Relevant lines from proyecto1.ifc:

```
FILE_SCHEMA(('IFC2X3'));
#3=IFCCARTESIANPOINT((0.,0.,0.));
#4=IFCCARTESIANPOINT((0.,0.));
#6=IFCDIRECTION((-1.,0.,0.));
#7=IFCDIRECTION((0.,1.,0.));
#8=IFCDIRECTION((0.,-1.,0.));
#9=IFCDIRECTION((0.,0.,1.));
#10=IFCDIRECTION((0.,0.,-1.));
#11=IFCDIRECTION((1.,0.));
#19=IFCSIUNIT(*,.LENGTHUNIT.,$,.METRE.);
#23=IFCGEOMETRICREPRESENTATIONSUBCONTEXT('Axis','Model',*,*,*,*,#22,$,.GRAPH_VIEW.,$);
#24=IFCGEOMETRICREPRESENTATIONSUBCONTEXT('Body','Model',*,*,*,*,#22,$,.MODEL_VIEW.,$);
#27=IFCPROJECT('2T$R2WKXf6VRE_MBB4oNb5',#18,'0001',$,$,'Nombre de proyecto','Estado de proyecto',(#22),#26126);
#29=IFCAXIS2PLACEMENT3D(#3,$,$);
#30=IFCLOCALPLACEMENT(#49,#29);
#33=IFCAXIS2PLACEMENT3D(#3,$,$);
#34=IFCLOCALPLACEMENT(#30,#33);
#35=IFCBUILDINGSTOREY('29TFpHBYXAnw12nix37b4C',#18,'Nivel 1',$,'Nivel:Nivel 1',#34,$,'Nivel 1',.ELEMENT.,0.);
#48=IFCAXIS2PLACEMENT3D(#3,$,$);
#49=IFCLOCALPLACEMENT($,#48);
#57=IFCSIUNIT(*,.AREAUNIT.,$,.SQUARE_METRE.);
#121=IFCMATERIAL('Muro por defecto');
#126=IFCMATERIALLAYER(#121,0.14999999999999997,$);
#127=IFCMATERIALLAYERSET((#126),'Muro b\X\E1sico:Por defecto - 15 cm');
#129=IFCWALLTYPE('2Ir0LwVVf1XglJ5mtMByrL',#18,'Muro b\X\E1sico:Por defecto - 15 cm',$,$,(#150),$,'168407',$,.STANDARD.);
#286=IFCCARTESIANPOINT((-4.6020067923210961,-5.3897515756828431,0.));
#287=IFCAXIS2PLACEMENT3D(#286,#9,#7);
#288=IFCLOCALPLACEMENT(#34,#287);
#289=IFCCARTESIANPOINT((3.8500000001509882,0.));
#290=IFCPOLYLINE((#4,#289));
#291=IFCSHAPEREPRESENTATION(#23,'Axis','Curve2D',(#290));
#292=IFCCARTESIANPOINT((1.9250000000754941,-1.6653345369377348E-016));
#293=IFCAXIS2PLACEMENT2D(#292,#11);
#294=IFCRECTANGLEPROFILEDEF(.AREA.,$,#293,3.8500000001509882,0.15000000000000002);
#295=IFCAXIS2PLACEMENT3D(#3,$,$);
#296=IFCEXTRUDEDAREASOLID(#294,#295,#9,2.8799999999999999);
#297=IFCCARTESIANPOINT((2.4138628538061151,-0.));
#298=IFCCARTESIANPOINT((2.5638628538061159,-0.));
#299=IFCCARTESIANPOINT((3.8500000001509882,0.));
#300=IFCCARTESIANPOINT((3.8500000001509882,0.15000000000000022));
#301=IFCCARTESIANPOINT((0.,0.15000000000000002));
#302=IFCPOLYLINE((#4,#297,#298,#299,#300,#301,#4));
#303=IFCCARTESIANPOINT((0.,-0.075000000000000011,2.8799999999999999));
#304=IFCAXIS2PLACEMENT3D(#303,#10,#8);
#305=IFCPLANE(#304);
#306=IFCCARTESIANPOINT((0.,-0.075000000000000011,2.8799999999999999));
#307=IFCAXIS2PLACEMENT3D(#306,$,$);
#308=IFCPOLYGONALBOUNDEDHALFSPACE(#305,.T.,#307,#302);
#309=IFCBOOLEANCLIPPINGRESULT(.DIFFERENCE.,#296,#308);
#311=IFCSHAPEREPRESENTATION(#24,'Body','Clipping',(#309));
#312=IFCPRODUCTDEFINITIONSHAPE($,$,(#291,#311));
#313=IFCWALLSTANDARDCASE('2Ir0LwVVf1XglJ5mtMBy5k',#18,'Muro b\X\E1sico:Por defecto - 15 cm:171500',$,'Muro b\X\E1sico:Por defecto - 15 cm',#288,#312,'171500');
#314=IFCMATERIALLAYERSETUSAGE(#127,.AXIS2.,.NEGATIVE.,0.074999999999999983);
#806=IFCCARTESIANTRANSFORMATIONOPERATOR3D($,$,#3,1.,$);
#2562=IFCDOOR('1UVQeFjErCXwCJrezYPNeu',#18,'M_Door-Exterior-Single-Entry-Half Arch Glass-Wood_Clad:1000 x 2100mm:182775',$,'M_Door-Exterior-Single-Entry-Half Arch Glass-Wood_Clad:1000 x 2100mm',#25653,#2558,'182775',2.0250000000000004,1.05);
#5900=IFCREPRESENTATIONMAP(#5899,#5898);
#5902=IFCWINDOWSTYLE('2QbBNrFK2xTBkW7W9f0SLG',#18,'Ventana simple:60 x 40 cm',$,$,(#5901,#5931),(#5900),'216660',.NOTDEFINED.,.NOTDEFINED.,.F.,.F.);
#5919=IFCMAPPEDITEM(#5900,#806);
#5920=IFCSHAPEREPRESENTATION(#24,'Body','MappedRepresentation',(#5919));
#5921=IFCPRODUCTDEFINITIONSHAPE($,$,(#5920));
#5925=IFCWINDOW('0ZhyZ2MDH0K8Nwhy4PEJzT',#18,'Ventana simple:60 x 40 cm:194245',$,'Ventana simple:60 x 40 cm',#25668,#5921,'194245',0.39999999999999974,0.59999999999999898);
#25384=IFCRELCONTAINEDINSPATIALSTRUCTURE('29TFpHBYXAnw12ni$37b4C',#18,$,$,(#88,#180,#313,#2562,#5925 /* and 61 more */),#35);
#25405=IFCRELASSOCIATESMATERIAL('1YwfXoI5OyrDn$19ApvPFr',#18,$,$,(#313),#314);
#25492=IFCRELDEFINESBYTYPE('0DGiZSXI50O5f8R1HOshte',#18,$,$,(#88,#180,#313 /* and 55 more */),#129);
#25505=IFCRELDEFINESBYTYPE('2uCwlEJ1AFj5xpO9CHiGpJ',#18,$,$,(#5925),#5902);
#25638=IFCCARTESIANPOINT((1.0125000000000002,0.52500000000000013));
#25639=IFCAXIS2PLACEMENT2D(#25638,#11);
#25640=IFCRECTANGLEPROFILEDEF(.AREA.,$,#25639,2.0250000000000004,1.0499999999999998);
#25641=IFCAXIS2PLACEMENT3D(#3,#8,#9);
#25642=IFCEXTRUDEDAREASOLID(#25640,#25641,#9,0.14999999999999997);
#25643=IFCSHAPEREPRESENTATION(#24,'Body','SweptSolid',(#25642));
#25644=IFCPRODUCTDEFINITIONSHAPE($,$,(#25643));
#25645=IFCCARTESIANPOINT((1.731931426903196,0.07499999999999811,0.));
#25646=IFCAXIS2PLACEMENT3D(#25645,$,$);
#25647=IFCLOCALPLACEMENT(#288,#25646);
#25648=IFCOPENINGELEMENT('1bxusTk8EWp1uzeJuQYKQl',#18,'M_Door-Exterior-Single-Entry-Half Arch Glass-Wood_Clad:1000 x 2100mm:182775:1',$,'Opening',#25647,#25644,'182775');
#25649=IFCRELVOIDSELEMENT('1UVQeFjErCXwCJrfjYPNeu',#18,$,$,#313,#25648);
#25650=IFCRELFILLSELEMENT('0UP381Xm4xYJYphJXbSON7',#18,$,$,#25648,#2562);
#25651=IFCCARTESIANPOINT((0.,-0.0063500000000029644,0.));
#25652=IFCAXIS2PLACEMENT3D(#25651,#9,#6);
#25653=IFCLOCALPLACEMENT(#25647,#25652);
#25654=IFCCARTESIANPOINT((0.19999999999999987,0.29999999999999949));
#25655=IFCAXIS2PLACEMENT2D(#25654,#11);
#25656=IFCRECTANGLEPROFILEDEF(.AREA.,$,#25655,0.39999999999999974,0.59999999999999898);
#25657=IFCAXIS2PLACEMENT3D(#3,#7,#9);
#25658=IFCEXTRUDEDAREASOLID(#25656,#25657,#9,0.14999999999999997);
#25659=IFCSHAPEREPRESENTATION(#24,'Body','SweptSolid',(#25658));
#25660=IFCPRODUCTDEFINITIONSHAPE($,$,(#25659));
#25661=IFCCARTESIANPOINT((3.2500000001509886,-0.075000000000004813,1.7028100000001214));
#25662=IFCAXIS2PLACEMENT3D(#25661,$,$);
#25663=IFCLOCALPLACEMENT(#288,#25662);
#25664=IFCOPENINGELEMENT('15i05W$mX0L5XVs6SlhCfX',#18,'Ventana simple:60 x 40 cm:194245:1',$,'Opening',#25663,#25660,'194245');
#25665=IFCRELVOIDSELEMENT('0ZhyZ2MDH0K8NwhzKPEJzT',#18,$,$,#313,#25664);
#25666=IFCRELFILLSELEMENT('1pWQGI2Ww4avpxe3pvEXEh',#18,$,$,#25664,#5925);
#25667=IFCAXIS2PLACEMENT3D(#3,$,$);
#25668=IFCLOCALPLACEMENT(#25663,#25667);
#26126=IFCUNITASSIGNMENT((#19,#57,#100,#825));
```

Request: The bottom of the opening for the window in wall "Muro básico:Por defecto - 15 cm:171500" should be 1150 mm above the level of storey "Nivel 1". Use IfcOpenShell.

```python
import numpy as np
import ifcopenshell
import ifcopenshell.api.geometry
import ifcopenshell.geom
import ifcopenshell.util.element
import ifcopenshell.util.placement
import ifcopenshell.util.shape
import ifcopenshell.util.unit

model = ifcopenshell.open("proyecto1.ifc")
unit_scale = ifcopenshell.util.unit.calculate_unit_scale(model)

window = model.by_id(5925)
opening = window.FillsVoids[0].RelatingOpeningElement
storey = ifcopenshell.util.element.get_container(window, ifc_class="IfcBuildingStorey")
level = ifcopenshell.util.placement.get_local_placement(storey.ObjectPlacement)[2, 3]

# The opening's origin need not be at the sill, so measure its lowest point.
shape = ifcopenshell.geom.create_shape(ifcopenshell.geom.settings(), opening)
bottom = ifcopenshell.util.shape.get_shape_bottom_elevation(shape, shape.geometry) / unit_scale
dz = level + 1.15 / unit_scale - bottom

shift = np.array([0.0, 0.0, dz])
# The window is placed relative to its opening, so it follows when the opening moves.
matrix = ifcopenshell.util.placement.get_local_placement(opening.ObjectPlacement)
matrix[:3, 3] += shift
ifcopenshell.api.geometry.edit_object_placement(
    model, product=opening, matrix=matrix, is_si=False, should_transform_children=True
)

print(f"moved by {dz * unit_scale:+.3f} m")

model.write("proyecto1_updated.ifc")
```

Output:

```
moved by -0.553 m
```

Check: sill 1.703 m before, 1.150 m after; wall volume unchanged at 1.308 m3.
